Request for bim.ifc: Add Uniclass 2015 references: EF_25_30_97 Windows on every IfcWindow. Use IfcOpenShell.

First a look at what the model holds.

```python
import ifcopenshell

model = ifcopenshell.open("bim.ifc")
print(model.schema)
print("classifications:", [c.Name for c in model.by_type("IfcClassification")])
for ifc_class in ("IfcDoor", "IfcRoof", "IfcStair", "IfcWall", "IfcWindow"):
    print(ifc_class, len(model.by_type(ifc_class)))
```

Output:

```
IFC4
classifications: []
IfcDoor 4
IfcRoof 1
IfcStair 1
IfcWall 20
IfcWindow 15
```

```python
import ifcopenshell
import ifcopenshell.api.classification

model = ifcopenshell.open("bim.ifc")

system = ifcopenshell.api.classification.add_classification(model, classification="Uniclass 2015")

codes = {
    "IfcWindow": ("EF_25_30_97", "Windows"),
}
for ifc_class, (code, name) in codes.items():
    products = model.by_type(ifc_class)
    ifcopenshell.api.classification.add_reference(
        model, products=products, classification=system, identification=code, name=name
    )
    print(code, len(products))

model.write("bim-out.ifc")
```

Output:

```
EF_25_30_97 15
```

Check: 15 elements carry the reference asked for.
